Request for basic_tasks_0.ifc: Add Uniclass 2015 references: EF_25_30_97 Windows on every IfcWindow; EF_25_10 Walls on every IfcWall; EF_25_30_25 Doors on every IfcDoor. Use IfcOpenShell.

First a look at what the model holds.

```python
import ifcopenshell

model = ifcopenshell.open("basic_tasks_0.ifc")
print(model.schema)
print("classifications:", [c.Name for c in model.by_type("IfcClassification")])
for ifc_class in ("IfcDoor", "IfcRoof", "IfcStair", "IfcWall", "IfcWindow"):
    print(ifc_class, len(model.by_type(ifc_class)))
```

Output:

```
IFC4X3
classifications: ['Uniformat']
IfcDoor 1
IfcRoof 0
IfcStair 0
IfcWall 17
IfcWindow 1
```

```python
import ifcopenshell
import ifcopenshell.api.classification

model = ifcopenshell.open("basic_tasks_0.ifc")

system = ifcopenshell.api.classification.add_classification(model, classification="Uniclass 2015")

codes = {
    "IfcWindow": ("EF_25_30_97", "Windows"),
    "IfcWall": ("EF_25_10", "Walls"),
    "IfcDoor": ("EF_25_30_25", "Doors"),
}
for ifc_class, (code, name) in codes.items():
    products = model.by_type(ifc_class)
    ifcopenshell.api.classification.add_reference(
        model, products=products, classification=system, identification=code, name=name
    )
    print(code, len(products))

model.write("basic_tasks_0_rev.ifc")
```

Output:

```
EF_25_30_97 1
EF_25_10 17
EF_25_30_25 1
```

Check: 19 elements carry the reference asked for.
